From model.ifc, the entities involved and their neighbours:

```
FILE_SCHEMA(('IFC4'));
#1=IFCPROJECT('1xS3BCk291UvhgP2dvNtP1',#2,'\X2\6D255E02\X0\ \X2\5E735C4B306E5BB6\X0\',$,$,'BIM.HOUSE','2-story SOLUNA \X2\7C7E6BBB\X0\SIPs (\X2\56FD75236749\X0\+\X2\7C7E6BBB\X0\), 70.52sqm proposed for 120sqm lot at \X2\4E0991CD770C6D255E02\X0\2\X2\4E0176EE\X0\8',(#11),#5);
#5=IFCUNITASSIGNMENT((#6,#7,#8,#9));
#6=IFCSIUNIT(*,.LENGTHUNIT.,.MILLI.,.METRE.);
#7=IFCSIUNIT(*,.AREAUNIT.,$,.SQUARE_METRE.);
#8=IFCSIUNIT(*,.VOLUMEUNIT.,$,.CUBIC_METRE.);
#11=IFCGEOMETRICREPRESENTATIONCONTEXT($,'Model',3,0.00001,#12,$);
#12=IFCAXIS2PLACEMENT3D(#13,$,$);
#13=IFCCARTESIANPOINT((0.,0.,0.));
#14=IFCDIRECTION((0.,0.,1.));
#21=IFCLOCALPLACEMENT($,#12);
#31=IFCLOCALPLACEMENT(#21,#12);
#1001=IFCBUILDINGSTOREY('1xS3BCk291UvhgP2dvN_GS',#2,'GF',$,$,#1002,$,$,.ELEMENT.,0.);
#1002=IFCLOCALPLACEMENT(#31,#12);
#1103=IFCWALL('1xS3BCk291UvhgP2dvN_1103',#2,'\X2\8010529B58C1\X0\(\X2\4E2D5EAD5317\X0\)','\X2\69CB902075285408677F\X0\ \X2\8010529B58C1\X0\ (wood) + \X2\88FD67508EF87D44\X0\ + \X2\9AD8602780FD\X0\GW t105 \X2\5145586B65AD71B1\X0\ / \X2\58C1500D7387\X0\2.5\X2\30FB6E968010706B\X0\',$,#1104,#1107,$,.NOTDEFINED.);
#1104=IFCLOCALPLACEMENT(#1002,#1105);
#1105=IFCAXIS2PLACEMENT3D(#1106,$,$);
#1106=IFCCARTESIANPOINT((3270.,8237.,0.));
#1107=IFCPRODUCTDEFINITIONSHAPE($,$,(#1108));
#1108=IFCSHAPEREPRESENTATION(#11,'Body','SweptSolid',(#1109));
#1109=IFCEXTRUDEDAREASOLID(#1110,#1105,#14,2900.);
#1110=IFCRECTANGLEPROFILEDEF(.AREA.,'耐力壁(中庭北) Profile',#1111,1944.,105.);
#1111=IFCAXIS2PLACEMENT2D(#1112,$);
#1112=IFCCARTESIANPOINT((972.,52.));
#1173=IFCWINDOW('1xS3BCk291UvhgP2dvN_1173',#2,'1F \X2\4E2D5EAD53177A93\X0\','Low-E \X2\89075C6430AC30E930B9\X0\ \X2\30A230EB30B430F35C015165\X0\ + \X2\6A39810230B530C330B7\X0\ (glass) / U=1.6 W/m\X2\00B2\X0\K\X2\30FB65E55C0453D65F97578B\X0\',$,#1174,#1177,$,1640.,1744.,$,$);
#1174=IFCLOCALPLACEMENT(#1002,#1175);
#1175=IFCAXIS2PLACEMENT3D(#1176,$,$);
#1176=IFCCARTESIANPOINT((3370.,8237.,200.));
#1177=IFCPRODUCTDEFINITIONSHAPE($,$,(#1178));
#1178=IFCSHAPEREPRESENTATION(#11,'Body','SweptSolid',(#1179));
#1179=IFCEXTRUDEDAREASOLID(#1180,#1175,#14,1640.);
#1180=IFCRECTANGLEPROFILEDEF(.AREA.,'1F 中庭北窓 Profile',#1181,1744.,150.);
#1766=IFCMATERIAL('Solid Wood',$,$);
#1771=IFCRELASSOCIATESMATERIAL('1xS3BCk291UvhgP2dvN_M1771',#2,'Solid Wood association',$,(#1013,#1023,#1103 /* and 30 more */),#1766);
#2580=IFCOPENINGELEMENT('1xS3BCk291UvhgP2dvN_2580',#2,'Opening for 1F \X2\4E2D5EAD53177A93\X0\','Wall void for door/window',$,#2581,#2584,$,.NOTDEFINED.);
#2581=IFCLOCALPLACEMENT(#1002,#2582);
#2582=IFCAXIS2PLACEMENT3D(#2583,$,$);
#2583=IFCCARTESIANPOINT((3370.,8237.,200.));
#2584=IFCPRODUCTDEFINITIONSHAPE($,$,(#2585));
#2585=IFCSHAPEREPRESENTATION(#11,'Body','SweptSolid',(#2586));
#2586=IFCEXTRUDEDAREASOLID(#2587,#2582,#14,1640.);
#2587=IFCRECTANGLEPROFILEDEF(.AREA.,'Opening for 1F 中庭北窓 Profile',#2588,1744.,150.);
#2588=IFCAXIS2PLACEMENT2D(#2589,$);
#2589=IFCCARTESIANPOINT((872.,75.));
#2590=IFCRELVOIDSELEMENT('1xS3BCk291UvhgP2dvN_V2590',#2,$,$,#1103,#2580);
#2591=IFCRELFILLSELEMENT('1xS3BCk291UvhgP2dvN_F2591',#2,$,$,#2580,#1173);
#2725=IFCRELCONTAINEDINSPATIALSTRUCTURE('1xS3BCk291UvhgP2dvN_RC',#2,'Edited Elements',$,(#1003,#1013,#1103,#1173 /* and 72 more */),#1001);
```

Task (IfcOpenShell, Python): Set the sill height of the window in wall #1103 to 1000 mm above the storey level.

```python
import numpy as np
import ifcopenshell
import ifcopenshell.api.geometry
import ifcopenshell.geom
import ifcopenshell.util.element
import ifcopenshell.util.placement
import ifcopenshell.util.shape
import ifcopenshell.util.unit

model = ifcopenshell.open("model.ifc")
unit_scale = ifcopenshell.util.unit.calculate_unit_scale(model)

window = model.by_guid("1xS3BCk291UvhgP2dvN_1173")
opening = window.FillsVoids[0].RelatingOpeningElement
storey = ifcopenshell.util.element.get_container(window, ifc_class="IfcBuildingStorey")
level = ifcopenshell.util.placement.get_local_placement(storey.ObjectPlacement)[2, 3]

# The opening's origin need not be at the sill, so measure its lowest point.
shape = ifcopenshell.geom.create_shape(ifcopenshell.geom.settings(), opening)
bottom = ifcopenshell.util.shape.get_shape_bottom_elevation(shape, shape.geometry) / unit_scale
dz = level + 1 / unit_scale - bottom

shift = np.array([0.0, 0.0, dz])
# The window is not placed relative to its opening, so move both.
for product in (opening, window):
    matrix = ifcopenshell.util.placement.get_local_placement(product.ObjectPlacement)
    matrix[:3, 3] += shift
    ifcopenshell.api.geometry.edit_object_placement(model, product=product, matrix=matrix, is_si=False)

print(f"moved by {dz * unit_scale:+.3f} m")

model.write("model_updated.ifc")
```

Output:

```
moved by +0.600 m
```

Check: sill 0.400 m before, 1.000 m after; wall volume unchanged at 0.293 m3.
